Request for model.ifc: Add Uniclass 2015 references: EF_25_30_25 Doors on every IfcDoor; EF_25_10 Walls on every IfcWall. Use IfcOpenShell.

First a look at what the model holds.

```python
import ifcopenshell

model = ifcopenshell.open("model.ifc")
print(model.schema)
print("classifications:", [c.Name for c in model.by_type("IfcClassification")])
for ifc_class in ("IfcDoor", "IfcRoof", "IfcStair", "IfcWall", "IfcWindow"):
    print(ifc_class, len(model.by_type(ifc_class)))
```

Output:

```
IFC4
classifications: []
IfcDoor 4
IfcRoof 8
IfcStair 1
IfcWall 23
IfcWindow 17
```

```python
import ifcopenshell
import ifcopenshell.api.classification

model = ifcopenshell.open("model.ifc")

system = ifcopenshell.api.classification.add_classification(model, classification="Uniclass 2015")

codes = {
    "IfcDoor": ("EF_25_30_25", "Doors"),
    "IfcWall": ("EF_25_10", "Walls"),
}
for ifc_class, (code, name) in codes.items():
    products = model.by_type(ifc_class)
    ifcopenshell.api.classification.add_reference(
        model, products=products, classification=system, identification=code, name=name
    )
    print(code, len(products))

model.write("model_rev.ifc")
```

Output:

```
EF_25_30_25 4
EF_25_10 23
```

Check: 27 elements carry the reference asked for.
